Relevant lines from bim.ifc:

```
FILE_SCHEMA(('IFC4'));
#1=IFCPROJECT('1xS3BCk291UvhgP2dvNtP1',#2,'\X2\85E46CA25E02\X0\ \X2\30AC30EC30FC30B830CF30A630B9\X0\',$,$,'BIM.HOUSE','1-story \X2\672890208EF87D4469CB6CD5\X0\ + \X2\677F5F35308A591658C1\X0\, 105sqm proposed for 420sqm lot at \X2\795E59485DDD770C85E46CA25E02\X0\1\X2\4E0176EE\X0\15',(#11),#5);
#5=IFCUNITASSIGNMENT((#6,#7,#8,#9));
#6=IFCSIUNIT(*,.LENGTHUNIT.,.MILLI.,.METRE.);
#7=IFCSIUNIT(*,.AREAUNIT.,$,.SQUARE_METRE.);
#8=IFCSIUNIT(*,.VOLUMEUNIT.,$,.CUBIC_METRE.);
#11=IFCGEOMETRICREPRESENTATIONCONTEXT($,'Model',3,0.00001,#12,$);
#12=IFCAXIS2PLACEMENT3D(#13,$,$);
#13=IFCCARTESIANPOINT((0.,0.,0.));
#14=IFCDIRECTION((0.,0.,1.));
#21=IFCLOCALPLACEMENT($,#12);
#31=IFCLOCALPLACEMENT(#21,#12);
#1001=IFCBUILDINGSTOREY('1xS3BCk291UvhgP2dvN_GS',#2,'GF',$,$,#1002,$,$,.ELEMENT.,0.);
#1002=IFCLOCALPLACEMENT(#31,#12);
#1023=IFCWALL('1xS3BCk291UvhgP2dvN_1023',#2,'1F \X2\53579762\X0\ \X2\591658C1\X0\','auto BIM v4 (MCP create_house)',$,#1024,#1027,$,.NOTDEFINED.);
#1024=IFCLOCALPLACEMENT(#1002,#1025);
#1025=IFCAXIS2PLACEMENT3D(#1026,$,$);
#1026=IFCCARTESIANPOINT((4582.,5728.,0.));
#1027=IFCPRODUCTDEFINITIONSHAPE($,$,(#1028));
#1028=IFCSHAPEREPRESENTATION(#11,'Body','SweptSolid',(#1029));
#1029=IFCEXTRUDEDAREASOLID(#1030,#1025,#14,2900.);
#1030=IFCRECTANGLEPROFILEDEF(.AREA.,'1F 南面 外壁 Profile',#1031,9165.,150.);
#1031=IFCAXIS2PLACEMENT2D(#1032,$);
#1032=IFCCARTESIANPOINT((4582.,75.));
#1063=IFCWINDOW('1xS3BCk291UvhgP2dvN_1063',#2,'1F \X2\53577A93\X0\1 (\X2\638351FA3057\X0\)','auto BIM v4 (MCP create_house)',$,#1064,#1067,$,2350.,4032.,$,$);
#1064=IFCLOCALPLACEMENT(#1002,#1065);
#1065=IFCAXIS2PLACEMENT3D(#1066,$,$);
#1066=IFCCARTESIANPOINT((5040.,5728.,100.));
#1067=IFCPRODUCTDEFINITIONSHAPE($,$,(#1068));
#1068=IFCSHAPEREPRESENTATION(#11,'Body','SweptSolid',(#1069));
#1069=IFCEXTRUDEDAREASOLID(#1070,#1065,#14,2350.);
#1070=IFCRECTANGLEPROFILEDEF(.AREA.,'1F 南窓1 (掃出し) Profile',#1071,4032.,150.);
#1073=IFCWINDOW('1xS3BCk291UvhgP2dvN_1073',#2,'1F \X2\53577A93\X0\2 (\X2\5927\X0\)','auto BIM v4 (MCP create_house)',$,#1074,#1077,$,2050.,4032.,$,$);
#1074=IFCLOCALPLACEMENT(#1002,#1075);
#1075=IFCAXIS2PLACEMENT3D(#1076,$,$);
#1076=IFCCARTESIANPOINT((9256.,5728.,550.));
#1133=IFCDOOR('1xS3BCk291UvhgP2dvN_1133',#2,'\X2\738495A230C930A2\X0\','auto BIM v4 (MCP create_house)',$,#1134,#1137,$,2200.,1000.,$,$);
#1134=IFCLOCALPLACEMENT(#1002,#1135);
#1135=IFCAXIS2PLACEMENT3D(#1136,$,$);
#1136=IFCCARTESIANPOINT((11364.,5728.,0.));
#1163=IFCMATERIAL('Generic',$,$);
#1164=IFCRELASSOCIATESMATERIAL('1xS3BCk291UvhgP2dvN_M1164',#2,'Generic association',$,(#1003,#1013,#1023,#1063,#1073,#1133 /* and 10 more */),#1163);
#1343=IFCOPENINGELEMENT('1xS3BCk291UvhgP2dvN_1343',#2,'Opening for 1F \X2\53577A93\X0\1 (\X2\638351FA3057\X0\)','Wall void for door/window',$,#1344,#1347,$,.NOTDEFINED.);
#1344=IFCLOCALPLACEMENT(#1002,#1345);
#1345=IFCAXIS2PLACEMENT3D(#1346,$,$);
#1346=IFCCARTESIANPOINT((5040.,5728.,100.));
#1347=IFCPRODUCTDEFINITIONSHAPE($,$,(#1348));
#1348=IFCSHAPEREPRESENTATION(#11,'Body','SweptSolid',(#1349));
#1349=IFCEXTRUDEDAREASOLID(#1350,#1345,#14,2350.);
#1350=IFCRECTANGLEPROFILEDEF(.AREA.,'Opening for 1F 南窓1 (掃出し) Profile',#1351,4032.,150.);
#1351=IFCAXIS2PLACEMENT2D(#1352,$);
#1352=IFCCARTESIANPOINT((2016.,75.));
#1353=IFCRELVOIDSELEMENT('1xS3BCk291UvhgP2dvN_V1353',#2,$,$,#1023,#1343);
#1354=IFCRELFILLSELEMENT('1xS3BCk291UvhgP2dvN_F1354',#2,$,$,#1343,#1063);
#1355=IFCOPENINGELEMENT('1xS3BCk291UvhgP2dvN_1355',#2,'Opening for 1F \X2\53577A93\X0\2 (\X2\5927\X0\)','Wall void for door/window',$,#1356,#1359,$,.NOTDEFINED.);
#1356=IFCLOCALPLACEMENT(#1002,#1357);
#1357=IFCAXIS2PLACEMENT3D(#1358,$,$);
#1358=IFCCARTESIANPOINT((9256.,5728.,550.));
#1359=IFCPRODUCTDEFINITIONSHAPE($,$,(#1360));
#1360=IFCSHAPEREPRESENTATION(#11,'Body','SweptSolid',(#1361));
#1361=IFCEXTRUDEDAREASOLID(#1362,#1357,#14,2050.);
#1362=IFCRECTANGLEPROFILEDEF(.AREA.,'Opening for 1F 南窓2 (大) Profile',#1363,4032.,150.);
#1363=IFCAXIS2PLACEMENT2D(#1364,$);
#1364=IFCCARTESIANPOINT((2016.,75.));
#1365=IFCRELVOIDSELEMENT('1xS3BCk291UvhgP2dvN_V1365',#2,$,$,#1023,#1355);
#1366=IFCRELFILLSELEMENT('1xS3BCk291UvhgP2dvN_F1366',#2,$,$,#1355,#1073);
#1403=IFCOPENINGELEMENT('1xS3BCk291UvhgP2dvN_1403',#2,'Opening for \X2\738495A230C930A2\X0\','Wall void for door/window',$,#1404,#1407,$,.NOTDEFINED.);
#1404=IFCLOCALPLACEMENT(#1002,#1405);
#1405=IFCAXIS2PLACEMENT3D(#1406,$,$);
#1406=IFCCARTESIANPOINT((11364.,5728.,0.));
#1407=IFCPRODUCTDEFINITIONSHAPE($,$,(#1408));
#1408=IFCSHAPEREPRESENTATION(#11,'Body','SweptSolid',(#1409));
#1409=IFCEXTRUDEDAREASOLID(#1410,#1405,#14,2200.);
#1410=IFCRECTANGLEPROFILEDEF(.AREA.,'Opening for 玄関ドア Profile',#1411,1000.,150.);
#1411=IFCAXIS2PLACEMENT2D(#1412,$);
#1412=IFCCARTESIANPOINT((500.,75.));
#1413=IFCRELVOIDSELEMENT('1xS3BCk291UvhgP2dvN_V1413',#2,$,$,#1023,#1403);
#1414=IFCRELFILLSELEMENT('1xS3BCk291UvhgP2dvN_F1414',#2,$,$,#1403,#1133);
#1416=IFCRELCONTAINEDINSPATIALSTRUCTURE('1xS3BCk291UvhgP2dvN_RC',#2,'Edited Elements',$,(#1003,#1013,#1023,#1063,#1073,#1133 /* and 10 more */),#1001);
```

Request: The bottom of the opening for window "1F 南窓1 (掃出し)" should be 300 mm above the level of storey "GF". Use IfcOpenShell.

```python
import numpy as np
import ifcopenshell
import ifcopenshell.api.geometry
import ifcopenshell.geom
import ifcopenshell.util.element
import ifcopenshell.util.placement
import ifcopenshell.util.shape
import ifcopenshell.util.unit

model = ifcopenshell.open("bim.ifc")
unit_scale = ifcopenshell.util.unit.calculate_unit_scale(model)

window = model.by_guid("1xS3BCk291UvhgP2dvN_1063")
opening = window.FillsVoids[0].RelatingOpeningElement
storey = ifcopenshell.util.element.get_container(window, ifc_class="IfcBuildingStorey")
level = ifcopenshell.util.placement.get_local_placement(storey.ObjectPlacement)[2, 3]

# The opening's origin need not be at the sill, so measure its lowest point.
shape = ifcopenshell.geom.create_shape(ifcopenshell.geom.settings(), opening)
bottom = ifcopenshell.util.shape.get_shape_bottom_elevation(shape, shape.geometry) / unit_scale
dz = level + 0.3 / unit_scale - bottom

shift = np.array([0.0, 0.0, dz])
# The window is not placed relative to its opening, so move both.
for product in (opening, window):
    matrix = ifcopenshell.util.placement.get_local_placement(product.ObjectPlacement)
    matrix[:3, 3] += shift
    ifcopenshell.api.geometry.edit_object_placement(model, product=product, matrix=matrix, is_si=False)

print(f"moved by {dz * unit_scale:+.3f} m")

model.write("bim-out.ifc")
```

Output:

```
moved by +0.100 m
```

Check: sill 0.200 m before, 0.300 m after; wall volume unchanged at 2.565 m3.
